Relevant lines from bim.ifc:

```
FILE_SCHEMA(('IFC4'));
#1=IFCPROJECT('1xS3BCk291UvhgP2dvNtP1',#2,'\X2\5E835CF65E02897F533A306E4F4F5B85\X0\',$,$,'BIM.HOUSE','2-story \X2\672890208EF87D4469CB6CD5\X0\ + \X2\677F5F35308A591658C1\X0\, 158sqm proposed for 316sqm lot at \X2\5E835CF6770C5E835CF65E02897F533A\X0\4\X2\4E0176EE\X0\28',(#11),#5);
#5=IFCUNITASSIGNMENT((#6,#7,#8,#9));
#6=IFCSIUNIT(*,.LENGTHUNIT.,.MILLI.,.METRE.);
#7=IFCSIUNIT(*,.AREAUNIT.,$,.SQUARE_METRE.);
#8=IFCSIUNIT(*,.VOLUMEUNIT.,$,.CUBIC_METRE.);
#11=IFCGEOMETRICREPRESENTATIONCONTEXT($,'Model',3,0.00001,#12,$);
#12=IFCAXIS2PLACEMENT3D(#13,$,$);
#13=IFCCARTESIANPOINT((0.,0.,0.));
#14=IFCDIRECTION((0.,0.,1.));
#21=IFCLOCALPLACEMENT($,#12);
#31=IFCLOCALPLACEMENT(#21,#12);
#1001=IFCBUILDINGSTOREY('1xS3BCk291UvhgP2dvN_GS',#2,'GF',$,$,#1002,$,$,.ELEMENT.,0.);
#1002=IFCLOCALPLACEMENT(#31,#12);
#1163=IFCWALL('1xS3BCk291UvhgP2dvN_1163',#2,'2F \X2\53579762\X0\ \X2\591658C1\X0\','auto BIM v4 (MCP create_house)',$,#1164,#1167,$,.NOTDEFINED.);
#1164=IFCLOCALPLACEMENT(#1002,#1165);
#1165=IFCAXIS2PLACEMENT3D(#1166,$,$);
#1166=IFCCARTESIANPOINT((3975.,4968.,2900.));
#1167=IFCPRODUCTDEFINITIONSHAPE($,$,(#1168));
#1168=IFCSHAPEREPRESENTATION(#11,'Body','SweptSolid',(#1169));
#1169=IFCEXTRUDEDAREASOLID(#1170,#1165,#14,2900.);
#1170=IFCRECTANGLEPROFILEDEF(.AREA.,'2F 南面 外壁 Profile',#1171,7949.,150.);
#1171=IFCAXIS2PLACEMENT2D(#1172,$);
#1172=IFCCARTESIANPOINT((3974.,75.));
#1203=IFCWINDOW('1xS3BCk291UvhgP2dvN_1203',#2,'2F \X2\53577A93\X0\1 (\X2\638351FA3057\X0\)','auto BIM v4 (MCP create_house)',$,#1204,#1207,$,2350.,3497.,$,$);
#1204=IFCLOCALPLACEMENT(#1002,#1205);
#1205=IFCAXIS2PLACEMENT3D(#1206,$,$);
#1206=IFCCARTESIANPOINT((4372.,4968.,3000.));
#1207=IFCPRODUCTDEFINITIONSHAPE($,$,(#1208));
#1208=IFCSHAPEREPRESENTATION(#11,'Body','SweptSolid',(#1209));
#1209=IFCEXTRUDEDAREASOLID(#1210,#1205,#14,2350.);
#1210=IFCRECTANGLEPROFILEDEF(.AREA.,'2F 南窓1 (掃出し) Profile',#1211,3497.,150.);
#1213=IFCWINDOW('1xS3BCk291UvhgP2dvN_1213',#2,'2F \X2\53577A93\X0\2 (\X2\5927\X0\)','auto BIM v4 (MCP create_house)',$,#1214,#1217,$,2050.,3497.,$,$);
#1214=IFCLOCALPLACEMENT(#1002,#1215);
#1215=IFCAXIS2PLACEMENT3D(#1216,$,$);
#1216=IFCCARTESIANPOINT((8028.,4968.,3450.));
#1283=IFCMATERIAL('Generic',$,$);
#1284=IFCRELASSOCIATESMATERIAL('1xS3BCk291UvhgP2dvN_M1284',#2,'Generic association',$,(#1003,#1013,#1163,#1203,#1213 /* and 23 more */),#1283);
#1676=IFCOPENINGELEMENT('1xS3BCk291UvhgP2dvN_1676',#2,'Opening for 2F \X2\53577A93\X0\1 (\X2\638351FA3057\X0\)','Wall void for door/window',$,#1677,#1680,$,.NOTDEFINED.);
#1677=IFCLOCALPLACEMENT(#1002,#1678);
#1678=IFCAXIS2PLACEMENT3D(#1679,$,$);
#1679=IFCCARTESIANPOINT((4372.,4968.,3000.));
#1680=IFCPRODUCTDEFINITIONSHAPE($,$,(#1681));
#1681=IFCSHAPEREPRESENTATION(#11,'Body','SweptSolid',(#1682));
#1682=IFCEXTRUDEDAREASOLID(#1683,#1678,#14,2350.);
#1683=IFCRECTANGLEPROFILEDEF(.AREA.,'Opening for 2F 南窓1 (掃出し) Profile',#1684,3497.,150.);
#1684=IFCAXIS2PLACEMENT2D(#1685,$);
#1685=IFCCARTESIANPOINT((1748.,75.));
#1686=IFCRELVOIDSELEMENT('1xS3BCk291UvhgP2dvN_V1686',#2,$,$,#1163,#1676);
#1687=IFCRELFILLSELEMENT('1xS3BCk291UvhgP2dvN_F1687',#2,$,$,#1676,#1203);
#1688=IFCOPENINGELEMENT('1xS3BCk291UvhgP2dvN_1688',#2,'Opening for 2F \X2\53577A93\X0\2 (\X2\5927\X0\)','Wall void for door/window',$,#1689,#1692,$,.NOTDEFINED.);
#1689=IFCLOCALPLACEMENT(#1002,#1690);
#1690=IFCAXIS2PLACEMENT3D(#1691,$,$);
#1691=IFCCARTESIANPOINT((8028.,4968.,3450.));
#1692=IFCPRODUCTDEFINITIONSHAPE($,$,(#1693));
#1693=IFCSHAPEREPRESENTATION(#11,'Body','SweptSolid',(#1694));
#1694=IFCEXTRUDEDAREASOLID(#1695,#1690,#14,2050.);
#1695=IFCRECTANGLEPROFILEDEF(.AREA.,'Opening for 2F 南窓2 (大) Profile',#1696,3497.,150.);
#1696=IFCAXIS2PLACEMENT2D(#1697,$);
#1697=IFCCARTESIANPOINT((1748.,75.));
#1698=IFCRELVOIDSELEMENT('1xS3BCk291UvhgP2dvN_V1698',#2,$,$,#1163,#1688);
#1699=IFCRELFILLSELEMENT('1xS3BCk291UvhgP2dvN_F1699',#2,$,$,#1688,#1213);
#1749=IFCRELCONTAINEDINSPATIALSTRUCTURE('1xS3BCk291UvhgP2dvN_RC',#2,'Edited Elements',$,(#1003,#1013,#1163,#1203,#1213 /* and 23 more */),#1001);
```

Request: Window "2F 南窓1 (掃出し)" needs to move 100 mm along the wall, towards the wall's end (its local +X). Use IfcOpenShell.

```python
import ifcopenshell
import ifcopenshell.api.geometry
import ifcopenshell.util.placement
import ifcopenshell.util.unit

model = ifcopenshell.open("bim.ifc")
unit_scale = ifcopenshell.util.unit.calculate_unit_scale(model)

window = model.by_guid("1xS3BCk291UvhgP2dvN_1203")
opening = window.FillsVoids[0].RelatingOpeningElement
wall = opening.VoidsElements[0].RelatingBuildingElement

wall_matrix = ifcopenshell.util.placement.get_local_placement(wall.ObjectPlacement)
shift = wall_matrix[:3, 0] * 0.1 / unit_scale
before = ifcopenshell.util.placement.get_local_placement(window.ObjectPlacement)[:3, 3].copy()

# The window is not placed relative to its opening, so move both.
for product in (opening, window):
    matrix = ifcopenshell.util.placement.get_local_placement(product.ObjectPlacement)
    matrix[:3, 3] += shift
    ifcopenshell.api.geometry.edit_object_placement(model, product=product, matrix=matrix, is_si=False)

after = ifcopenshell.util.placement.get_local_placement(window.ObjectPlacement)[:3, 3]
print("window moved by", (after - before).round(3) + 0.0)

model.write("bim_rev.ifc")
```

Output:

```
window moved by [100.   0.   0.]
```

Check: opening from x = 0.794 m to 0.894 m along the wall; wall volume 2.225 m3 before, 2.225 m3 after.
